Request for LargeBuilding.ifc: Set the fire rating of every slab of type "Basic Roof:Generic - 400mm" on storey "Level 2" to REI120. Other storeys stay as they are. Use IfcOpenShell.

First a look at what the model holds.

```python
import ifcopenshell
import ifcopenshell.util.element

model = ifcopenshell.open("LargeBuilding.ifc")
print(model.schema)
storey = next(s for s in model.by_type("IfcBuildingStorey") if s.Name == "Level 2")
slabs = [e for e in ifcopenshell.util.element.get_decomposition(storey) if e.is_a("IfcSlab")]
seen = {}
for e in slabs:
    element_type = ifcopenshell.util.element.get_type(e)
    key = (element_type.Name if element_type != e and element_type else None, ifcopenshell.util.element.get_pset(e, "Pset_SlabCommon", "FireRating"))
    seen[key] = seen.get(key, 0) + 1
for (name, value), count in sorted(seen.items(), key=str):
    print(count, "x", name, "|", value)
```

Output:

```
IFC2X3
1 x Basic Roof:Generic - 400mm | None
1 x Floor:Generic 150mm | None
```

```python
import ifcopenshell
import ifcopenshell.api.pset
import ifcopenshell.util.element

model = ifcopenshell.open("LargeBuilding.ifc")

storey = next(s for s in model.by_type("IfcBuildingStorey") if s.Name == "Level 2")
slabs = [e for e in ifcopenshell.util.element.get_decomposition(storey) if e.is_a("IfcSlab")]

count = 0
for e in slabs:
    element_type = ifcopenshell.util.element.get_type(e)
    if element_type in (None, e) or element_type.Name != "Basic Roof:Generic - 400mm":
        continue
    # add_pset returns the element's existing set when there is one.
    pset = ifcopenshell.api.pset.add_pset(model, product=e, name="Pset_SlabCommon")
    ifcopenshell.api.pset.edit_pset(model, pset=pset, properties={"FireRating": "REI120"})
    count += 1

print(count, "slabs updated")

model.write("LargeBuilding_edited.ifc")
```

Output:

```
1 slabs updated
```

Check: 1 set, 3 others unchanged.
